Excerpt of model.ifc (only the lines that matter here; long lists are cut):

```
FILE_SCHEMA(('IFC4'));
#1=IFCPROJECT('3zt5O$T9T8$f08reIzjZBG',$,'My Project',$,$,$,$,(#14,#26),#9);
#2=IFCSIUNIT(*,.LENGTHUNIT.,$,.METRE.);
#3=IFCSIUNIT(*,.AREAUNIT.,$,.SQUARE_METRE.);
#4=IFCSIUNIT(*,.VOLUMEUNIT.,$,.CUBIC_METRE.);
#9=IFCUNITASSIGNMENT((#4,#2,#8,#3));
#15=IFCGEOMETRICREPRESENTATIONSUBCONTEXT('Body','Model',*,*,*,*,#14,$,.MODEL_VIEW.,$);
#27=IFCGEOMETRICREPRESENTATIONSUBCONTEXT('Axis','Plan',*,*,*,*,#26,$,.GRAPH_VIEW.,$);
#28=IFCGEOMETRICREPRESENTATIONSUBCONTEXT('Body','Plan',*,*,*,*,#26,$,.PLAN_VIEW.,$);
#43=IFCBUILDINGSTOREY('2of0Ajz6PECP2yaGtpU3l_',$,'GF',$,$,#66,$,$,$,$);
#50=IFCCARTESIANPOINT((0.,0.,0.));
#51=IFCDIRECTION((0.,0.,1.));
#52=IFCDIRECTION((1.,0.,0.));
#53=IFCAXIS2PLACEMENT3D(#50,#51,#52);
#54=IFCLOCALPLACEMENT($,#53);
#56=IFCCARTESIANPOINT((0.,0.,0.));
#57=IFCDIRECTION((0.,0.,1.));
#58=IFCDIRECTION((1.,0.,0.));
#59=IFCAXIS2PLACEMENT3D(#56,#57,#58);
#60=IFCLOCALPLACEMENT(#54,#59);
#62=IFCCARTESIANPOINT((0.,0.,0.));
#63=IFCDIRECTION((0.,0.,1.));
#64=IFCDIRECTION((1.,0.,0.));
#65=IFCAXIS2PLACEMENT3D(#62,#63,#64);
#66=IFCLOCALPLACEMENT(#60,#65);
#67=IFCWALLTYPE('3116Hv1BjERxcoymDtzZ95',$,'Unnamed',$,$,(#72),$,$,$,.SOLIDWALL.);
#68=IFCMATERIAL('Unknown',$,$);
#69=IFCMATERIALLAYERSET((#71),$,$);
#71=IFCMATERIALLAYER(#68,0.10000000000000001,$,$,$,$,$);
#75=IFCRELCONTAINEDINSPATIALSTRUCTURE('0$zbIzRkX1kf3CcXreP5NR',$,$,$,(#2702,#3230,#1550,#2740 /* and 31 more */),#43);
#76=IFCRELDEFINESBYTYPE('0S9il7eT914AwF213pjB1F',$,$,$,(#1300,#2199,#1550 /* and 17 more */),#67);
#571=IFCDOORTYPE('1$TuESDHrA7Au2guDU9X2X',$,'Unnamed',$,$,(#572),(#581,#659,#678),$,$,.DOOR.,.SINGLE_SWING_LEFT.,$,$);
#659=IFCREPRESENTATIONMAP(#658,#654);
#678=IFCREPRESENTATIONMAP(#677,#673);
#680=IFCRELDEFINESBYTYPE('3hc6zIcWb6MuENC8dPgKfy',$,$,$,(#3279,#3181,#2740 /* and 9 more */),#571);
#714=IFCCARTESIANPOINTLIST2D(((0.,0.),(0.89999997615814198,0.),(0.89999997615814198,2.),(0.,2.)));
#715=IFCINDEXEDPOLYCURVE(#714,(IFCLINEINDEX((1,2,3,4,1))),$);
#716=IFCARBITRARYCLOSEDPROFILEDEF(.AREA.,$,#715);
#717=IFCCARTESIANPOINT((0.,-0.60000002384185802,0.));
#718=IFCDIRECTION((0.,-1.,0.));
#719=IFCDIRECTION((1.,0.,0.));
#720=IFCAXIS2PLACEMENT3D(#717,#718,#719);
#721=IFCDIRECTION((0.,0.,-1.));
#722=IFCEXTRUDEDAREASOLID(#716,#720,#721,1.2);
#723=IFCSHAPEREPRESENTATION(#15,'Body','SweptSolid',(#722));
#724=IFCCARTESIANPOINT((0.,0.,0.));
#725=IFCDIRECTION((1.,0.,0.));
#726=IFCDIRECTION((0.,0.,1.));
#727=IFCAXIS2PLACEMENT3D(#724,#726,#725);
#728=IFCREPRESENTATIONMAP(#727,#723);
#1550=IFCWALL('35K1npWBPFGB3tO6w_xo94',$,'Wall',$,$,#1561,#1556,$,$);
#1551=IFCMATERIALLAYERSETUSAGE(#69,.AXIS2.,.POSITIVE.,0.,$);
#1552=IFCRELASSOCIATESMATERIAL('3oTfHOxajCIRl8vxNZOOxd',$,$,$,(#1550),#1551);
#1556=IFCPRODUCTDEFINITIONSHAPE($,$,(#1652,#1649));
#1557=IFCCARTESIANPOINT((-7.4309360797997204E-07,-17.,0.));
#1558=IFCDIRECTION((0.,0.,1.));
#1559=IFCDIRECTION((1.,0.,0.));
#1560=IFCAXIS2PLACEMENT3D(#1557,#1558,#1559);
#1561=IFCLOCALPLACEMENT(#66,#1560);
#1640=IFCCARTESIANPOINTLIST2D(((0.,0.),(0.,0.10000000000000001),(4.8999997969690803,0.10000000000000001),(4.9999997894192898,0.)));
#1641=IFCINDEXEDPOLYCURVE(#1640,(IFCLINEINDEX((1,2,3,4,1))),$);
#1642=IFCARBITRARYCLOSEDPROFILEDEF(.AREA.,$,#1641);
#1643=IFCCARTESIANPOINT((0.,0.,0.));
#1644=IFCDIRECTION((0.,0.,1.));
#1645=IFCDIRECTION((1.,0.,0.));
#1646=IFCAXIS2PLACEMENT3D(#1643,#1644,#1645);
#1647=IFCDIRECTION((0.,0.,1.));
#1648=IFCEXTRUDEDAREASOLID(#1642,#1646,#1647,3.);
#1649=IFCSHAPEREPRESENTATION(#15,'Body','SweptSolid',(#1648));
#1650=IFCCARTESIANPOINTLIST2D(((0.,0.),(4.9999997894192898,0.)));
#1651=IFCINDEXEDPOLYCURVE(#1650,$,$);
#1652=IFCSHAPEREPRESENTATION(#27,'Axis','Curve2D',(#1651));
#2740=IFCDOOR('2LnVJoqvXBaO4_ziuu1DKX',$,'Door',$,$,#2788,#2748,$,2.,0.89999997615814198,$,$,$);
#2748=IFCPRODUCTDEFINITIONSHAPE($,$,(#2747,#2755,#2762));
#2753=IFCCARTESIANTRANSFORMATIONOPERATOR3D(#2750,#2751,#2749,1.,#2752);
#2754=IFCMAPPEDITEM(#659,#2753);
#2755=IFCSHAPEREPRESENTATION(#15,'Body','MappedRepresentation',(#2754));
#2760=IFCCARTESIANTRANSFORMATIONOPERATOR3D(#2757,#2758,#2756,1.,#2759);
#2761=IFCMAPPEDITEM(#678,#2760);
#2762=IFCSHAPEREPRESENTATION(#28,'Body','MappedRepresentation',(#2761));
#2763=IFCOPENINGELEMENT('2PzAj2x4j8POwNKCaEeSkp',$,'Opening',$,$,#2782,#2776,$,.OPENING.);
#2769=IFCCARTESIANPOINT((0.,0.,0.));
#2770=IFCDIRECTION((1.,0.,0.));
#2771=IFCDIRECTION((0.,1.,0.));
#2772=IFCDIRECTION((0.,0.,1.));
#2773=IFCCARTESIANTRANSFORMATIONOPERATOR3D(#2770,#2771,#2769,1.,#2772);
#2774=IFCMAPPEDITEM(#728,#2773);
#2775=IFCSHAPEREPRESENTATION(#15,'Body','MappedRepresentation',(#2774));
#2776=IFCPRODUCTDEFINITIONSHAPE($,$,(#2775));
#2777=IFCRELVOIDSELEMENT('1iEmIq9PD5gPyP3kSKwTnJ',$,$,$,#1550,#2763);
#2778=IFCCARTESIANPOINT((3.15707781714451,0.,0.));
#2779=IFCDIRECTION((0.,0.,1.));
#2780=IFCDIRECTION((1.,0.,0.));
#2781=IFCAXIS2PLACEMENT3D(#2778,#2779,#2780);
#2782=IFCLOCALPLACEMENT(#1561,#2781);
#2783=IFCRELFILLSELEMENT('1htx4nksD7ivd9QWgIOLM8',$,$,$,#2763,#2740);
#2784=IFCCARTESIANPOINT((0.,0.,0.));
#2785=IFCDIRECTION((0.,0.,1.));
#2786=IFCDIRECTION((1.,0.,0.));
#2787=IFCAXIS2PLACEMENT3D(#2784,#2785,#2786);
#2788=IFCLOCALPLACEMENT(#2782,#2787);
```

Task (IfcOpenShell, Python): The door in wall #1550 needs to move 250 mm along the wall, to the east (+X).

```python
import ifcopenshell
import ifcopenshell.api.geometry
import ifcopenshell.util.placement
import ifcopenshell.util.unit

model = ifcopenshell.open("model.ifc")
unit_scale = ifcopenshell.util.unit.calculate_unit_scale(model)

door = model.by_guid("2LnVJoqvXBaO4_ziuu1DKX")
opening = door.FillsVoids[0].RelatingOpeningElement
wall = opening.VoidsElements[0].RelatingBuildingElement

wall_matrix = ifcopenshell.util.placement.get_local_placement(wall.ObjectPlacement)
shift = wall_matrix[:3, 0] * 0.25 / unit_scale
before = ifcopenshell.util.placement.get_local_placement(door.ObjectPlacement)[:3, 3].copy()

# The door is placed relative to its opening, so it follows when the opening moves.
matrix = ifcopenshell.util.placement.get_local_placement(opening.ObjectPlacement)
matrix[:3, 3] += shift
ifcopenshell.api.geometry.edit_object_placement(
    model, product=opening, matrix=matrix, is_si=False, should_transform_children=True
)

after = ifcopenshell.util.placement.get_local_placement(door.ObjectPlacement)[:3, 3]
print("door moved by", (after - before).round(3) + 0.0)

model.write("model-out.ifc")
```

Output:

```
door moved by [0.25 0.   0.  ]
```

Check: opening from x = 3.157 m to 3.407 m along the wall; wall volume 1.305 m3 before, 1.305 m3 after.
